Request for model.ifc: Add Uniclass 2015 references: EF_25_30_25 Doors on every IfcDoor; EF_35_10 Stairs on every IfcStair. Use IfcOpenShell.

First a look at what the model holds.

```python
import ifcopenshell

model = ifcopenshell.open("model.ifc")
print(model.schema)
print("classifications:", [c.Name for c in model.by_type("IfcClassification")])
for ifc_class in ("IfcDoor", "IfcRoof", "IfcStair", "IfcWall", "IfcWindow"):
    print(ifc_class, len(model.by_type(ifc_class)))
```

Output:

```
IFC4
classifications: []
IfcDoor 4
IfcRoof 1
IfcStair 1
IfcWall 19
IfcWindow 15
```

```python
import ifcopenshell
import ifcopenshell.api.classification

model = ifcopenshell.open("model.ifc")

system = ifcopenshell.api.classification.add_classification(model, classification="Uniclass 2015")

codes = {
    "IfcDoor": ("EF_25_30_25", "Doors"),
    "IfcStair": ("EF_35_10", "Stairs"),
}
for ifc_class, (code, name) in codes.items():
    products = model.by_type(ifc_class)
    ifcopenshell.api.classification.add_reference(
        model, products=products, classification=system, identification=code, name=name
    )
    print(code, len(products))

model.write("model_v2.ifc")
```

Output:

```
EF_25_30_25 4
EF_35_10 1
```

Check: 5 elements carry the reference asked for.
